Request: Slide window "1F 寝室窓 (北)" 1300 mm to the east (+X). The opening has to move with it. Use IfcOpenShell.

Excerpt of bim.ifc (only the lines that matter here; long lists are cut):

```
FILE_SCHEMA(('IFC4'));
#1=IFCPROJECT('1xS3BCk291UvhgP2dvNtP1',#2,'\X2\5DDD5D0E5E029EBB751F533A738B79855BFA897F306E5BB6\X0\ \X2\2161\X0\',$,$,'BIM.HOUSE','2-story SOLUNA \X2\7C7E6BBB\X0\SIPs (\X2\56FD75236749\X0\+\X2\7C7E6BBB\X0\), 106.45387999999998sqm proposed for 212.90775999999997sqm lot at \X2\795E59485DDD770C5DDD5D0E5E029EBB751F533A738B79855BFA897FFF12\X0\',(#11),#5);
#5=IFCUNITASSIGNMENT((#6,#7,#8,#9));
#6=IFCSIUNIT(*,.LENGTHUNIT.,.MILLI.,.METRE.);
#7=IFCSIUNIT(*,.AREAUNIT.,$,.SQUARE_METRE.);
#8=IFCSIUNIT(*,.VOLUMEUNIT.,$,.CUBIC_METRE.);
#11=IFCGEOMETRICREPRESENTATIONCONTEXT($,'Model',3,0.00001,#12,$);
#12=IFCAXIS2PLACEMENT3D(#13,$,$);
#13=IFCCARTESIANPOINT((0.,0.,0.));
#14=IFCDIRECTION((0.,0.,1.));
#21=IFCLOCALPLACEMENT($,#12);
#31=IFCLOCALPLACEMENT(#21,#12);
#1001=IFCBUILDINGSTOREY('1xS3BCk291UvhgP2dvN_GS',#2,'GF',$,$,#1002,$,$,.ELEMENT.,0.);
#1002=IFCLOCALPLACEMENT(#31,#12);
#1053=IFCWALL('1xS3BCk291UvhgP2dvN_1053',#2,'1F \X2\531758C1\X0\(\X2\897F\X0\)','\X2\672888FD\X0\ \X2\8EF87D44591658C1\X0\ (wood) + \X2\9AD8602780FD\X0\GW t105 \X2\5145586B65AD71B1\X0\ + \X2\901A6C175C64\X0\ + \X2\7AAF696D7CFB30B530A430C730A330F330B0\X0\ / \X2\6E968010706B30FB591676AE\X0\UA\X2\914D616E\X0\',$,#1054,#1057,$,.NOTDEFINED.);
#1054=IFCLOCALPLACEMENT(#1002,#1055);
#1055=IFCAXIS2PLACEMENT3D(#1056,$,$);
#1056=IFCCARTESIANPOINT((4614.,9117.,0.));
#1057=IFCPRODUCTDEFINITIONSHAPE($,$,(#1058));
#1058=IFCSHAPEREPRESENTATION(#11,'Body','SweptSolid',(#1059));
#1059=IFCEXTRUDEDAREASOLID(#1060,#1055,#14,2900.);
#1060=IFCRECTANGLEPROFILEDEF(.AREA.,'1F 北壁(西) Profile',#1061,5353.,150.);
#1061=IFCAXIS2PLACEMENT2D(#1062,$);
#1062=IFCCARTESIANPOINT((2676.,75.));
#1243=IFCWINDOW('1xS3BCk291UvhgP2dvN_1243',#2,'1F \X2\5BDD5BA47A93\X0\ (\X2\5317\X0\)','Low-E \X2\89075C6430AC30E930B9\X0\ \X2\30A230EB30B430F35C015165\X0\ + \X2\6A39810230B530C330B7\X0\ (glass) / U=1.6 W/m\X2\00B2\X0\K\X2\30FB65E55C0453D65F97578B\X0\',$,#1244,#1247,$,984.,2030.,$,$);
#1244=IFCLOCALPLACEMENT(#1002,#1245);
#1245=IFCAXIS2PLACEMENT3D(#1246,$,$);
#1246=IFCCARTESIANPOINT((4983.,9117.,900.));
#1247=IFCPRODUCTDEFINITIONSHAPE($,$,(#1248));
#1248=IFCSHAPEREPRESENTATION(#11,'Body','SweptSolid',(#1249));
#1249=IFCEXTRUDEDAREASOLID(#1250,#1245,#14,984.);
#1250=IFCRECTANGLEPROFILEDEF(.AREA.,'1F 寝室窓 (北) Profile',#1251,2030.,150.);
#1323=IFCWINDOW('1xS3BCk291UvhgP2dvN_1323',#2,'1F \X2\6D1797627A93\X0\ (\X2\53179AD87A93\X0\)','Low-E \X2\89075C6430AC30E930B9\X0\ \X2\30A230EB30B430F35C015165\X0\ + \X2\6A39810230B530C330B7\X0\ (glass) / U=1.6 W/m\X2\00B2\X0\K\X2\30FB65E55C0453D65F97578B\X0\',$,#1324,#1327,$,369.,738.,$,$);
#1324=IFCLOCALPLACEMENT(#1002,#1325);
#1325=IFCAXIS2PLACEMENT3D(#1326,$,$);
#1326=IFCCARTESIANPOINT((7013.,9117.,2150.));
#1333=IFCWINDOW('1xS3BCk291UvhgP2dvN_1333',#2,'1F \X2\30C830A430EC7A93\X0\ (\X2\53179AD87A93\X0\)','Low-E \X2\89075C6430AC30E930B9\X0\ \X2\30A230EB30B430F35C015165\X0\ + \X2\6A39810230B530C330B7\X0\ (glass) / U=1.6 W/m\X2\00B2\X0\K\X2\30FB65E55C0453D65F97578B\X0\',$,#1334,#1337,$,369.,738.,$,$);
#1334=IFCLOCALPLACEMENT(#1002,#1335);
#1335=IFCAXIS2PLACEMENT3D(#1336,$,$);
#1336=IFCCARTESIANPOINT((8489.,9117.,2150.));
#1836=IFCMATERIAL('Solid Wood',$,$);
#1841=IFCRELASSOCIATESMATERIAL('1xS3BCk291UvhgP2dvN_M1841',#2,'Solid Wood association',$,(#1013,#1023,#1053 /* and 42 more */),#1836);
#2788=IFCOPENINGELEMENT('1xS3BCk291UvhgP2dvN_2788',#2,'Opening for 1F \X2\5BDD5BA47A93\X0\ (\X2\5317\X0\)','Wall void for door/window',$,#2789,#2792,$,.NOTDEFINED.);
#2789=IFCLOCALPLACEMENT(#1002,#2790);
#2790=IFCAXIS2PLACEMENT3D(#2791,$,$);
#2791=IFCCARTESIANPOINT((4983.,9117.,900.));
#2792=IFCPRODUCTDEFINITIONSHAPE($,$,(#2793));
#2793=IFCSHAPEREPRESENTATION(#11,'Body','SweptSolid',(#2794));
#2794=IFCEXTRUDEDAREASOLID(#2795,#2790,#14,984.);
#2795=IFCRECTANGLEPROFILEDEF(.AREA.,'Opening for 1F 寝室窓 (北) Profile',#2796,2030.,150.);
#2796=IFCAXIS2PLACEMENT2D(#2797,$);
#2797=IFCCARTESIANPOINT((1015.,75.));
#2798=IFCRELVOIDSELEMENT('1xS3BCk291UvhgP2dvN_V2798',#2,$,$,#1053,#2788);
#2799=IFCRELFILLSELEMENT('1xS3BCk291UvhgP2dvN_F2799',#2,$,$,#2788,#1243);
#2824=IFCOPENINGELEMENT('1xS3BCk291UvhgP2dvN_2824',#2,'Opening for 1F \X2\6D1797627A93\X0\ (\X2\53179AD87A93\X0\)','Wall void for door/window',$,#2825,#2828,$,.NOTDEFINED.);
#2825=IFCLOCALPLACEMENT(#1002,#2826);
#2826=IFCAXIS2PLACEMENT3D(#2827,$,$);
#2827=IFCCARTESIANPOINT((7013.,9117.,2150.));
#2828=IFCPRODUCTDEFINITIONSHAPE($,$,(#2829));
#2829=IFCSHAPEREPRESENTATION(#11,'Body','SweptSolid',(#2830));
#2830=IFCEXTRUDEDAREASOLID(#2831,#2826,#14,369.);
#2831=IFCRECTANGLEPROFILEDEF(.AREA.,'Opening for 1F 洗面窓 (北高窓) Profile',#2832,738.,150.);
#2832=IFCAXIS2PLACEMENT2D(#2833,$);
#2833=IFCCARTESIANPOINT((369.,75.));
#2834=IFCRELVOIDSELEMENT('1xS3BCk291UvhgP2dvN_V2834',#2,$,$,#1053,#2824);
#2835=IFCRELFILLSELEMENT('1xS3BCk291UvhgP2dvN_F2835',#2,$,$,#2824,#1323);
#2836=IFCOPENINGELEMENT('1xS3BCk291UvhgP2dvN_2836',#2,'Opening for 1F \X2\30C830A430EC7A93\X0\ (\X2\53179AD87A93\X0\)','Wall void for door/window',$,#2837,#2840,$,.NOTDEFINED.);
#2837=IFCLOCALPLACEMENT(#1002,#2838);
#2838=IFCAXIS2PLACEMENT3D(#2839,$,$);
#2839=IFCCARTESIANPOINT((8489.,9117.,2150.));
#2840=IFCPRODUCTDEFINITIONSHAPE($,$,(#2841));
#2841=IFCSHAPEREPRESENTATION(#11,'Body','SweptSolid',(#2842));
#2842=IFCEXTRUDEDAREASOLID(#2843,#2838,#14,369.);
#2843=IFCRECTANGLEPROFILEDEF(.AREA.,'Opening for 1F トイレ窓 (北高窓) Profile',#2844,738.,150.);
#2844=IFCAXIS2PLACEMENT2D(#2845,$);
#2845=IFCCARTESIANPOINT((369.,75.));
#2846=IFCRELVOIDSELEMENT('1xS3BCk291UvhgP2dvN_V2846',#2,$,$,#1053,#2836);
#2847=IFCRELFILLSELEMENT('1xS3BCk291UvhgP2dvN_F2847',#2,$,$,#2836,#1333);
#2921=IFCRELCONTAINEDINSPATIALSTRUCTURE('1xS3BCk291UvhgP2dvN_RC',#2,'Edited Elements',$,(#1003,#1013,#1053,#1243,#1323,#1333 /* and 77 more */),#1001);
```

```python
import ifcopenshell
import ifcopenshell.api.geometry
import ifcopenshell.util.placement
import ifcopenshell.util.unit

model = ifcopenshell.open("bim.ifc")
unit_scale = ifcopenshell.util.unit.calculate_unit_scale(model)

window = model.by_id(1243)
opening = window.FillsVoids[0].RelatingOpeningElement
wall = opening.VoidsElements[0].RelatingBuildingElement

wall_matrix = ifcopenshell.util.placement.get_local_placement(wall.ObjectPlacement)
shift = wall_matrix[:3, 0] * 1.3 / unit_scale
before = ifcopenshell.util.placement.get_local_placement(window.ObjectPlacement)[:3, 3].copy()

# The window is not placed relative to its opening, so move both.
for product in (opening, window):
    matrix = ifcopenshell.util.placement.get_local_placement(product.ObjectPlacement)
    matrix[:3, 3] += shift
    ifcopenshell.api.geometry.edit_object_placement(model, product=product, matrix=matrix, is_si=False)

after = ifcopenshell.util.placement.get_local_placement(window.ObjectPlacement)[:3, 3]
print("window moved by", (after - before).round(3) + 0.0)

model.write("bim_rev.ifc")
```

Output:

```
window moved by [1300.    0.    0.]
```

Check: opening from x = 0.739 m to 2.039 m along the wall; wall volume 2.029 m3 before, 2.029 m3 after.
